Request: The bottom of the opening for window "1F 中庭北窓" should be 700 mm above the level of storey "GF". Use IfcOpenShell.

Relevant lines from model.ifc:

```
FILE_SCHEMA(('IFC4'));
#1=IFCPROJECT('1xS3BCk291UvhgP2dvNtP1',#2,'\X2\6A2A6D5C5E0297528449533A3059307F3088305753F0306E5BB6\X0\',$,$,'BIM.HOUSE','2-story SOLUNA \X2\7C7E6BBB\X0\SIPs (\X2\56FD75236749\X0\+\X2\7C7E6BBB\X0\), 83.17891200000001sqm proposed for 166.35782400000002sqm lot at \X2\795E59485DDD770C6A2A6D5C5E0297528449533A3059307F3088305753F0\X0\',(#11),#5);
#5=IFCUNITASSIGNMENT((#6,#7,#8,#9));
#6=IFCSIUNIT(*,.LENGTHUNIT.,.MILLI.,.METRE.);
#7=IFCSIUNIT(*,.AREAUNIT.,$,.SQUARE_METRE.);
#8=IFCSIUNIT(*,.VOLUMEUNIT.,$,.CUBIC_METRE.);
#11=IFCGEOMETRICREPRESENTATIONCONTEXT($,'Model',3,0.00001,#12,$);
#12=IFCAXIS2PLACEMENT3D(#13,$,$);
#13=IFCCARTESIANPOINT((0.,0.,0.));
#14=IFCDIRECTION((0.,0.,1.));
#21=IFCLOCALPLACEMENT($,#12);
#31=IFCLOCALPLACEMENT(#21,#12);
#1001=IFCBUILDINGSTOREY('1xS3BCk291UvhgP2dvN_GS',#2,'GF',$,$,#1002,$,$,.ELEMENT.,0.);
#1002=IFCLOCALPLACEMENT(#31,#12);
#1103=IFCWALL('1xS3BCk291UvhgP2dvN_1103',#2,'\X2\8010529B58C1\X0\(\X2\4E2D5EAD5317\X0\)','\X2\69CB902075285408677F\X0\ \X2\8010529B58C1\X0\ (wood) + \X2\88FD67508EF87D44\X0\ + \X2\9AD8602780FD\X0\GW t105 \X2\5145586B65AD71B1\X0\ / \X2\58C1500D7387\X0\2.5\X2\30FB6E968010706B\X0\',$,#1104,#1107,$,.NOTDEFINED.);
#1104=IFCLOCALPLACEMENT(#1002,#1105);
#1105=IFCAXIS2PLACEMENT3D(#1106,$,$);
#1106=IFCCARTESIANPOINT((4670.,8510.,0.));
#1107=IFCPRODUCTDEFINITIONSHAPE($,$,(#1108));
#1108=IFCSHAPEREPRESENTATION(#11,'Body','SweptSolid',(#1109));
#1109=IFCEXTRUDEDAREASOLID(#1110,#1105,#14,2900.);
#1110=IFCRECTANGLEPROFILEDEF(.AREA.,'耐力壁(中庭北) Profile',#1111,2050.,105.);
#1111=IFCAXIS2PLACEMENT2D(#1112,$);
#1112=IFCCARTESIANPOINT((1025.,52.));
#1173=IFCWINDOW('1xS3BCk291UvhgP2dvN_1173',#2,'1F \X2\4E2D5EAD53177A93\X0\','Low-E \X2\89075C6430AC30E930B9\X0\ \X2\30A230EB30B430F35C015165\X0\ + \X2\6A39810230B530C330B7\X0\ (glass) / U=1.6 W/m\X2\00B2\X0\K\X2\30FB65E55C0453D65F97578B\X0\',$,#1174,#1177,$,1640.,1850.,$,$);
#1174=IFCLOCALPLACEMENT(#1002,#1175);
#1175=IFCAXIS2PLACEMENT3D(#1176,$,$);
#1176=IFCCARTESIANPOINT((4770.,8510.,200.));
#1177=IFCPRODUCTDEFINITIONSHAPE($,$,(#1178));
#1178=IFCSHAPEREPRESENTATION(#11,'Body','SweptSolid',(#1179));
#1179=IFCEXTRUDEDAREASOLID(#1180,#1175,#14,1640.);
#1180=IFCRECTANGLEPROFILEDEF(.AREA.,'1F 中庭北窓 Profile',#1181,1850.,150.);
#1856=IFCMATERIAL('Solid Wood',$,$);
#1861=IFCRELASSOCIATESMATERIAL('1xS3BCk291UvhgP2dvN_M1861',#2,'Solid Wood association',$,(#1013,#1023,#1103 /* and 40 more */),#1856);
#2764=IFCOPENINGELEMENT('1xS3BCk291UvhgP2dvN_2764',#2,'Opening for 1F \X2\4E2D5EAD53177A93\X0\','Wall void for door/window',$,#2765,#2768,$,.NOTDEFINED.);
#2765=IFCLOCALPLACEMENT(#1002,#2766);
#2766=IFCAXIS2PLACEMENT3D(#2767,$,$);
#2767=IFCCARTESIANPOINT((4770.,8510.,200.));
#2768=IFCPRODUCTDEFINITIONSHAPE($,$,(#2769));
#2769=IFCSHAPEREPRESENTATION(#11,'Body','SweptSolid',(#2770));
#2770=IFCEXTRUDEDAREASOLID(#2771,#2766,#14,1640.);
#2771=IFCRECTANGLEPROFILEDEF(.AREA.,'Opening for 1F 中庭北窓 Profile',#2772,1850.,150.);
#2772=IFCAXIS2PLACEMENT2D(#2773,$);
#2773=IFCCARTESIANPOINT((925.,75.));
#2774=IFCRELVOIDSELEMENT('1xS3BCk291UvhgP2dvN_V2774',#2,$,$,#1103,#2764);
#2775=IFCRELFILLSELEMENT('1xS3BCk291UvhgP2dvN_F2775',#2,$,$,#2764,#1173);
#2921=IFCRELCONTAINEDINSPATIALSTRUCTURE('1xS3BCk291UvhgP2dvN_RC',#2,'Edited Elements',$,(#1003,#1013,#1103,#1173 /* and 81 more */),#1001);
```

```python
import numpy as np
import ifcopenshell
import ifcopenshell.api.geometry
import ifcopenshell.geom
import ifcopenshell.util.element
import ifcopenshell.util.placement
import ifcopenshell.util.shape
import ifcopenshell.util.unit

model = ifcopenshell.open("model.ifc")
unit_scale = ifcopenshell.util.unit.calculate_unit_scale(model)

window = model.by_guid("1xS3BCk291UvhgP2dvN_1173")
opening = window.FillsVoids[0].RelatingOpeningElement
storey = ifcopenshell.util.element.get_container(window, ifc_class="IfcBuildingStorey")
level = ifcopenshell.util.placement.get_local_placement(storey.ObjectPlacement)[2, 3]

# The opening's origin need not be at the sill, so measure its lowest point.
shape = ifcopenshell.geom.create_shape(ifcopenshell.geom.settings(), opening)
bottom = ifcopenshell.util.shape.get_shape_bottom_elevation(shape, shape.geometry) / unit_scale
dz = level + 0.7 / unit_scale - bottom

shift = np.array([0.0, 0.0, dz])
# The window is not placed relative to its opening, so move both.
for product in (opening, window):
    matrix = ifcopenshell.util.placement.get_local_placement(product.ObjectPlacement)
    matrix[:3, 3] += shift
    ifcopenshell.api.geometry.edit_object_placement(model, product=product, matrix=matrix, is_si=False)

print(f"moved by {dz * unit_scale:+.3f} m")

model.write("model_v2.ifc")
```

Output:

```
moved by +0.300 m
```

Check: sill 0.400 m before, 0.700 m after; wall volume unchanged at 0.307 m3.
